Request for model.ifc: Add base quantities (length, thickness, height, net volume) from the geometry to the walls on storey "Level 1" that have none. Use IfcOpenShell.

First a look at what the model holds.

```python
import ifcopenshell
import ifcopenshell.util.element
import ifcopenshell.util.unit

model = ifcopenshell.open("model.ifc")
print(model.schema)
for unit_type in ("LENGTHUNIT", "AREAUNIT", "VOLUMEUNIT"):
    print(unit_type, ifcopenshell.util.unit.calculate_unit_scale(model, unit_type))
storey = next(s for s in model.by_type("IfcBuildingStorey") if s.Name == "Level 1")
walls = [e for e in ifcopenshell.util.element.get_decomposition(storey) if e.is_a("IfcWall")]
for e in sorted(walls, key=lambda e: e.id()):
    print(e.id(), e.is_a(), e.Name, list(ifcopenshell.util.element.get_psets(e, qtos_only=True)), sep=" | ")
```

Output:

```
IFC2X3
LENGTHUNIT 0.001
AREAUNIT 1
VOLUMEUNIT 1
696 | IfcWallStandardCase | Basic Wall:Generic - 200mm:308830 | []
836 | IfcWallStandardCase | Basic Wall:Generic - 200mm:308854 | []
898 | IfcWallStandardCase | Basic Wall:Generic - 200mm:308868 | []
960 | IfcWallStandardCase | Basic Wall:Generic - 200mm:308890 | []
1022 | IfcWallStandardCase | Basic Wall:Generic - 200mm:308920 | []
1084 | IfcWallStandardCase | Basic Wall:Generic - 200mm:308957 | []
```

```python
import ifcopenshell
import ifcopenshell.api.pset
import ifcopenshell.geom
import ifcopenshell.util.element
import ifcopenshell.util.shape
import ifcopenshell.util.unit

model = ifcopenshell.open("model.ifc")
unit_scale = ifcopenshell.util.unit.calculate_unit_scale(model)
volume_scale = ifcopenshell.util.unit.calculate_unit_scale(model, "VOLUMEUNIT")
settings = ifcopenshell.geom.settings()

storey = next(s for s in model.by_type("IfcBuildingStorey") if s.Name == "Level 1")
walls = [e for e in ifcopenshell.util.element.get_decomposition(storey) if e.is_a("IfcWall")]

for e in sorted(walls, key=lambda e: e.id()):
    if ifcopenshell.util.element.get_psets(e, qtos_only=True, should_inherit=False):
        continue
    # Geometry comes back in metres, in the element's own axes.
    shape = ifcopenshell.geom.create_shape(settings, e)
    values = {
        "Length": ifcopenshell.util.shape.get_x(shape.geometry) / unit_scale,
        "Width": ifcopenshell.util.shape.get_y(shape.geometry) / unit_scale,
        "Height": ifcopenshell.util.shape.get_z(shape.geometry) / unit_scale,
        "NetVolume": ifcopenshell.util.shape.get_volume(shape.geometry) / volume_scale,
    }
    qto = ifcopenshell.api.pset.add_qto(model, product=e, name="BaseQuantities")
    ifcopenshell.api.pset.edit_qto(model, qto=qto, properties=values)
    print(e.id(), {k: round(v, 3) for k, v in values.items()})

model.write("model_updated.ifc")
```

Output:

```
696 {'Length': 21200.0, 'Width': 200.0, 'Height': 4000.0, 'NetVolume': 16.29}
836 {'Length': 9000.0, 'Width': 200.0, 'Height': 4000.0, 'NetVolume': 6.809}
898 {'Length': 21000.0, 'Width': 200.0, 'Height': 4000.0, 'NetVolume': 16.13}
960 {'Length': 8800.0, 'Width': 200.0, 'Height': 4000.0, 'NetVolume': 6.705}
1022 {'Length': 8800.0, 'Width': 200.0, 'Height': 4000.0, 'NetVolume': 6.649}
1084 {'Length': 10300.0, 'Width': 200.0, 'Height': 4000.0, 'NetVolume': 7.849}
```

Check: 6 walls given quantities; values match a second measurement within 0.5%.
